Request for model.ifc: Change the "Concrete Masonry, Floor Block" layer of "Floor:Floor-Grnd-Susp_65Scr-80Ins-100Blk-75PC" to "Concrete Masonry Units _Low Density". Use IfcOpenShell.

First a look at what the model holds.

```python
import ifcopenshell
import ifcopenshell.util.element

model = ifcopenshell.open("model.ifc")
print(model.schema)
for layer_set in model.by_type("IfcMaterialLayerSet"):
    if layer_set.LayerSetName == "Floor:Floor-Grnd-Susp_65Scr-80Ins-100Blk-75PC":
        for layer in layer_set.MaterialLayers:
            print(layer.id(), layer.Material and layer.Material.Name, layer.LayerThickness, sep=" | ")
        print(len(ifcopenshell.util.element.get_elements_by_material(model, layer_set)), "elements and types use it")
print(sorted(m.Name for m in model.by_type("IfcMaterial") if m.Name)[:60])
```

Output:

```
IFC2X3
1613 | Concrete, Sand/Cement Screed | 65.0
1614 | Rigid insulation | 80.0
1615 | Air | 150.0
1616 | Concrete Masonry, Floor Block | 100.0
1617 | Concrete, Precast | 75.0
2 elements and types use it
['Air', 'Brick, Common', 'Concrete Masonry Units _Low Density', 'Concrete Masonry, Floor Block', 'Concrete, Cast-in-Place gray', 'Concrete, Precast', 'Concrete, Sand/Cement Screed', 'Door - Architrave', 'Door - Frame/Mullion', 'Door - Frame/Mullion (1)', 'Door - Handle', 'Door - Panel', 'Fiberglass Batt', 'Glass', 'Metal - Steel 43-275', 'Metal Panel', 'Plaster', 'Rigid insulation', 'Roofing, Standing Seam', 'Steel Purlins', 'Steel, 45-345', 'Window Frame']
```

```python
import ifcopenshell
import ifcopenshell.api.material

model = ifcopenshell.open("model.ifc")

layer_set = next(s for s in model.by_type("IfcMaterialLayerSet") if s.LayerSetName == "Floor:Floor-Grnd-Susp_65Scr-80Ins-100Blk-75PC")
layer = next(l for l in layer_set.MaterialLayers if l.Material and l.Material.Name == "Concrete Masonry, Floor Block")
material = next(m for m in model.by_type("IfcMaterial") if m.Name == "Concrete Masonry Units _Low Density")

# Point this one layer at the other material; renaming the old one would change it everywhere.
ifcopenshell.api.material.edit_layer(model, layer=layer, attributes={}, material=material)

print([l.Material.Name if l.Material else None for l in layer_set.MaterialLayers])

model.write("model_updated.ifc")
```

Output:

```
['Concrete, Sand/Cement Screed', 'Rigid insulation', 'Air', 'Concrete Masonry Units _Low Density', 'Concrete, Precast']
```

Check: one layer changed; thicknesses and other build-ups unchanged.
